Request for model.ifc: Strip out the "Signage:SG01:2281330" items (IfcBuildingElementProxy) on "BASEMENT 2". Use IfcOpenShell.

First a look at what the model holds.

```python
import ifcopenshell
import ifcopenshell.util.element

model = ifcopenshell.open("model.ifc")
print(model.schema)
storey = next(s for s in model.by_type("IfcBuildingStorey") if s.Name == "BASEMENT 2")
proxies = [e for e in ifcopenshell.util.element.get_decomposition(storey) if e.is_a("IfcBuildingElementProxy")]
seen = {}
for e in proxies:
    element_type = ifcopenshell.util.element.get_type(e)
    name = element_type.Name if element_type not in (None, e) else None
    seen[name] = seen.get(name, 0) + 1
for name, count in sorted(seen.items(), key=str):
    print(count, "x", name)
```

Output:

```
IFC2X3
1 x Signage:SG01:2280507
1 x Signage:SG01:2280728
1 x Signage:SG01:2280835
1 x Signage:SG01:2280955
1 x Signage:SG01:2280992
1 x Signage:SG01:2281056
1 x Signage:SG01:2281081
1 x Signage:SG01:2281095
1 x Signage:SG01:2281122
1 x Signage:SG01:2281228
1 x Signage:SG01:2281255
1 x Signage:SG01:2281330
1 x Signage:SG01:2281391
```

```python
import ifcopenshell
import ifcopenshell.api.root
import ifcopenshell.util.element

model = ifcopenshell.open("model.ifc")

storey = next(s for s in model.by_type("IfcBuildingStorey") if s.Name == "BASEMENT 2")
proxies = [e for e in ifcopenshell.util.element.get_decomposition(storey) if e.is_a("IfcBuildingElementProxy")]
targets = [e for e in proxies if (t := ifcopenshell.util.element.get_type(e)) not in (None, e) and t.Name == "Signage:SG01:2281330"]

for e in targets:
    ifcopenshell.api.root.remove_product(model, product=e)
print(len(targets), "removed")

model.write("model_updated.ifc")
```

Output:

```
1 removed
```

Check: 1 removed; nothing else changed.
